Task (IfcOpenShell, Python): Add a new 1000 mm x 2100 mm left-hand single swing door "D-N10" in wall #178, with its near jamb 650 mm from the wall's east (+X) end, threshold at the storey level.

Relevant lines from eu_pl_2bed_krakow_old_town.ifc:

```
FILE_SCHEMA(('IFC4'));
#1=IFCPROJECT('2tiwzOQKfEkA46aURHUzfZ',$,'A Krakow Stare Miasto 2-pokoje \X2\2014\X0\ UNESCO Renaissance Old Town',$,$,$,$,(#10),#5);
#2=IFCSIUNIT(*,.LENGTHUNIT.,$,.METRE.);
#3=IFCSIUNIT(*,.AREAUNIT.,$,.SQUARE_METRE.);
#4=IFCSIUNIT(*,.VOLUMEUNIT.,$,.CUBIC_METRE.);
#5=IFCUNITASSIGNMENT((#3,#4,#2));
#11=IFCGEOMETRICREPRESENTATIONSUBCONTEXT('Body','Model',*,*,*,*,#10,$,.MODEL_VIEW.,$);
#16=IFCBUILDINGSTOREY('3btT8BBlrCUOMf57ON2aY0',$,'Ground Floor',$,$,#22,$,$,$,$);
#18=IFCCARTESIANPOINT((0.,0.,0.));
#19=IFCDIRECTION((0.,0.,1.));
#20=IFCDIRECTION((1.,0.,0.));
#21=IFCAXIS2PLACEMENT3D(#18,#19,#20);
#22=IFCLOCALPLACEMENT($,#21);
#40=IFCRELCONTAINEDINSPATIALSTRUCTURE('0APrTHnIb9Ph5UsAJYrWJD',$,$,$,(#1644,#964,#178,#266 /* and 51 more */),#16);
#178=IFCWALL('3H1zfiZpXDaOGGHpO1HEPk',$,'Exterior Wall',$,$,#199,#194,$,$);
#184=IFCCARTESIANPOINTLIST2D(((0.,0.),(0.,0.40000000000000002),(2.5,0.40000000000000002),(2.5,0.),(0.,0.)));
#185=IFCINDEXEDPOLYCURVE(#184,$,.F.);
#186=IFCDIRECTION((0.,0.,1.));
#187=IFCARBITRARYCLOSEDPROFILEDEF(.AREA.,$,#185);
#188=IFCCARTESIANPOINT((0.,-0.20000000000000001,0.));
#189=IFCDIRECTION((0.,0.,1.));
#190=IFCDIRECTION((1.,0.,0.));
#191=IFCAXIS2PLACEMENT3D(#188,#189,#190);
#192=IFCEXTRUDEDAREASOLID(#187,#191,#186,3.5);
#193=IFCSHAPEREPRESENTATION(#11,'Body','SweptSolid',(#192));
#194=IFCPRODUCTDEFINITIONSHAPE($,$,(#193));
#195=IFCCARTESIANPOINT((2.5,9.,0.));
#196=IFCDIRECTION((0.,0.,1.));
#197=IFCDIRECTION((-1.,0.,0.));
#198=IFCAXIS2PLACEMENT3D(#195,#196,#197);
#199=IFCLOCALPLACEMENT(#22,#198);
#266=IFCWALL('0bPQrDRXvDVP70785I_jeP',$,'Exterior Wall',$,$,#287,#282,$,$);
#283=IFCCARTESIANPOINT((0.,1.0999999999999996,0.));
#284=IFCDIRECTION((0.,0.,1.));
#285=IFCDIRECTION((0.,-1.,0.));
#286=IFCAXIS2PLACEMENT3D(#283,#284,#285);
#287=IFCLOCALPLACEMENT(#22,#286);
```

```python
import numpy as np
import ifcopenshell
import ifcopenshell.api.feature
import ifcopenshell.api.geometry
import ifcopenshell.api.root
import ifcopenshell.api.spatial
import ifcopenshell.geom
import ifcopenshell.util.element
import ifcopenshell.util.placement
import ifcopenshell.util.representation
import ifcopenshell.util.shape
import ifcopenshell.util.unit

model = ifcopenshell.open("eu_pl_2bed_krakow_old_town.ifc")
unit_scale = ifcopenshell.util.unit.calculate_unit_scale(model)
settings = ifcopenshell.geom.settings()


def volume(element):
    """Net volume in cubic metres, openings subtracted."""
    shape = ifcopenshell.geom.create_shape(settings, element)
    return ifcopenshell.util.shape.get_volume(shape.geometry)


wall = model.by_guid("3H1zfiZpXDaOGGHpO1HEPk")
storey = ifcopenshell.util.element.get_container(wall, ifc_class="IfcBuildingStorey")
context = ifcopenshell.util.representation.get_context(model, "Model", "Body", "MODEL_VIEW")
before = volume(wall)

width, height, from_end, sill = 1, 2.1, 0.65, 0.0  # metres

# The wall runs along its own X axis, and the end named is its -X end.
wall_shape = ifcopenshell.geom.create_shape(settings, wall)
x, y, z = ifcopenshell.util.shape.get_vertices(wall_shape.geometry).T
start = x.min() + from_end
face, thickness = float(y.min()), float(y.max() - y.min())
wall_matrix = ifcopenshell.util.placement.get_local_placement(wall.ObjectPlacement)
level = ifcopenshell.util.placement.get_local_placement(storey.ObjectPlacement)[2, 3]


def in_wall(x, y):
    """Placement at x, y metres in the wall's axes, at sill height."""
    matrix = wall_matrix.copy()
    matrix[:, 3] = wall_matrix @ np.array([x / unit_scale, y / unit_scale, 0.0, 1.0])
    matrix[2, 3] = level + sill / unit_scale
    return matrix


# Opening: a box that overshoots both wall faces by 50 mm.
opening = ifcopenshell.api.root.create_entity(model, ifc_class="IfcOpeningElement", predefined_type="OPENING")
box = ifcopenshell.api.geometry.add_wall_representation(
    model, context=context, length=width, height=height, thickness=thickness + 0.1
)
ifcopenshell.api.geometry.assign_representation(model, product=opening, representation=box)
ifcopenshell.api.geometry.edit_object_placement(model, product=opening, matrix=in_wall(start, face - 0.05), is_si=False)
ifcopenshell.api.feature.add_feature(model, feature=opening, element=wall)

door = ifcopenshell.api.root.create_entity(model, ifc_class="IfcDoor", name="D-N10", predefined_type="DOOR")
door.OverallWidth, door.OverallHeight = width / unit_scale, height / unit_scale
door.OperationType = "SINGLE_SWING_LEFT"
body = ifcopenshell.api.geometry.add_door_representation(
    model,
    context=context,
    overall_width=door.OverallWidth,
    overall_height=door.OverallHeight,
    operation_type="SINGLE_SWING_LEFT",
    lining_properties={"LiningDepth": thickness / unit_scale, "ThresholdDepth": thickness / unit_scale},
)
ifcopenshell.api.geometry.assign_representation(model, product=door, representation=body)
ifcopenshell.api.spatial.assign_container(model, products=[door], relating_structure=storey)
ifcopenshell.api.feature.add_filling(model, opening=opening, element=door)

# The lining spans the wall, so the door starts at the wall face.
ifcopenshell.api.geometry.edit_object_placement(model, product=door, matrix=in_wall(start, face), is_si=False)

after = volume(wall)

print(f"wall volume {before:.3f} -> {after:.3f} m3")

model.write("eu_pl_2bed_krakow_old_town_updated.ifc")
```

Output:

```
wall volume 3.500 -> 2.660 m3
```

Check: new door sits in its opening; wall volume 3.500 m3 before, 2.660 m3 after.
